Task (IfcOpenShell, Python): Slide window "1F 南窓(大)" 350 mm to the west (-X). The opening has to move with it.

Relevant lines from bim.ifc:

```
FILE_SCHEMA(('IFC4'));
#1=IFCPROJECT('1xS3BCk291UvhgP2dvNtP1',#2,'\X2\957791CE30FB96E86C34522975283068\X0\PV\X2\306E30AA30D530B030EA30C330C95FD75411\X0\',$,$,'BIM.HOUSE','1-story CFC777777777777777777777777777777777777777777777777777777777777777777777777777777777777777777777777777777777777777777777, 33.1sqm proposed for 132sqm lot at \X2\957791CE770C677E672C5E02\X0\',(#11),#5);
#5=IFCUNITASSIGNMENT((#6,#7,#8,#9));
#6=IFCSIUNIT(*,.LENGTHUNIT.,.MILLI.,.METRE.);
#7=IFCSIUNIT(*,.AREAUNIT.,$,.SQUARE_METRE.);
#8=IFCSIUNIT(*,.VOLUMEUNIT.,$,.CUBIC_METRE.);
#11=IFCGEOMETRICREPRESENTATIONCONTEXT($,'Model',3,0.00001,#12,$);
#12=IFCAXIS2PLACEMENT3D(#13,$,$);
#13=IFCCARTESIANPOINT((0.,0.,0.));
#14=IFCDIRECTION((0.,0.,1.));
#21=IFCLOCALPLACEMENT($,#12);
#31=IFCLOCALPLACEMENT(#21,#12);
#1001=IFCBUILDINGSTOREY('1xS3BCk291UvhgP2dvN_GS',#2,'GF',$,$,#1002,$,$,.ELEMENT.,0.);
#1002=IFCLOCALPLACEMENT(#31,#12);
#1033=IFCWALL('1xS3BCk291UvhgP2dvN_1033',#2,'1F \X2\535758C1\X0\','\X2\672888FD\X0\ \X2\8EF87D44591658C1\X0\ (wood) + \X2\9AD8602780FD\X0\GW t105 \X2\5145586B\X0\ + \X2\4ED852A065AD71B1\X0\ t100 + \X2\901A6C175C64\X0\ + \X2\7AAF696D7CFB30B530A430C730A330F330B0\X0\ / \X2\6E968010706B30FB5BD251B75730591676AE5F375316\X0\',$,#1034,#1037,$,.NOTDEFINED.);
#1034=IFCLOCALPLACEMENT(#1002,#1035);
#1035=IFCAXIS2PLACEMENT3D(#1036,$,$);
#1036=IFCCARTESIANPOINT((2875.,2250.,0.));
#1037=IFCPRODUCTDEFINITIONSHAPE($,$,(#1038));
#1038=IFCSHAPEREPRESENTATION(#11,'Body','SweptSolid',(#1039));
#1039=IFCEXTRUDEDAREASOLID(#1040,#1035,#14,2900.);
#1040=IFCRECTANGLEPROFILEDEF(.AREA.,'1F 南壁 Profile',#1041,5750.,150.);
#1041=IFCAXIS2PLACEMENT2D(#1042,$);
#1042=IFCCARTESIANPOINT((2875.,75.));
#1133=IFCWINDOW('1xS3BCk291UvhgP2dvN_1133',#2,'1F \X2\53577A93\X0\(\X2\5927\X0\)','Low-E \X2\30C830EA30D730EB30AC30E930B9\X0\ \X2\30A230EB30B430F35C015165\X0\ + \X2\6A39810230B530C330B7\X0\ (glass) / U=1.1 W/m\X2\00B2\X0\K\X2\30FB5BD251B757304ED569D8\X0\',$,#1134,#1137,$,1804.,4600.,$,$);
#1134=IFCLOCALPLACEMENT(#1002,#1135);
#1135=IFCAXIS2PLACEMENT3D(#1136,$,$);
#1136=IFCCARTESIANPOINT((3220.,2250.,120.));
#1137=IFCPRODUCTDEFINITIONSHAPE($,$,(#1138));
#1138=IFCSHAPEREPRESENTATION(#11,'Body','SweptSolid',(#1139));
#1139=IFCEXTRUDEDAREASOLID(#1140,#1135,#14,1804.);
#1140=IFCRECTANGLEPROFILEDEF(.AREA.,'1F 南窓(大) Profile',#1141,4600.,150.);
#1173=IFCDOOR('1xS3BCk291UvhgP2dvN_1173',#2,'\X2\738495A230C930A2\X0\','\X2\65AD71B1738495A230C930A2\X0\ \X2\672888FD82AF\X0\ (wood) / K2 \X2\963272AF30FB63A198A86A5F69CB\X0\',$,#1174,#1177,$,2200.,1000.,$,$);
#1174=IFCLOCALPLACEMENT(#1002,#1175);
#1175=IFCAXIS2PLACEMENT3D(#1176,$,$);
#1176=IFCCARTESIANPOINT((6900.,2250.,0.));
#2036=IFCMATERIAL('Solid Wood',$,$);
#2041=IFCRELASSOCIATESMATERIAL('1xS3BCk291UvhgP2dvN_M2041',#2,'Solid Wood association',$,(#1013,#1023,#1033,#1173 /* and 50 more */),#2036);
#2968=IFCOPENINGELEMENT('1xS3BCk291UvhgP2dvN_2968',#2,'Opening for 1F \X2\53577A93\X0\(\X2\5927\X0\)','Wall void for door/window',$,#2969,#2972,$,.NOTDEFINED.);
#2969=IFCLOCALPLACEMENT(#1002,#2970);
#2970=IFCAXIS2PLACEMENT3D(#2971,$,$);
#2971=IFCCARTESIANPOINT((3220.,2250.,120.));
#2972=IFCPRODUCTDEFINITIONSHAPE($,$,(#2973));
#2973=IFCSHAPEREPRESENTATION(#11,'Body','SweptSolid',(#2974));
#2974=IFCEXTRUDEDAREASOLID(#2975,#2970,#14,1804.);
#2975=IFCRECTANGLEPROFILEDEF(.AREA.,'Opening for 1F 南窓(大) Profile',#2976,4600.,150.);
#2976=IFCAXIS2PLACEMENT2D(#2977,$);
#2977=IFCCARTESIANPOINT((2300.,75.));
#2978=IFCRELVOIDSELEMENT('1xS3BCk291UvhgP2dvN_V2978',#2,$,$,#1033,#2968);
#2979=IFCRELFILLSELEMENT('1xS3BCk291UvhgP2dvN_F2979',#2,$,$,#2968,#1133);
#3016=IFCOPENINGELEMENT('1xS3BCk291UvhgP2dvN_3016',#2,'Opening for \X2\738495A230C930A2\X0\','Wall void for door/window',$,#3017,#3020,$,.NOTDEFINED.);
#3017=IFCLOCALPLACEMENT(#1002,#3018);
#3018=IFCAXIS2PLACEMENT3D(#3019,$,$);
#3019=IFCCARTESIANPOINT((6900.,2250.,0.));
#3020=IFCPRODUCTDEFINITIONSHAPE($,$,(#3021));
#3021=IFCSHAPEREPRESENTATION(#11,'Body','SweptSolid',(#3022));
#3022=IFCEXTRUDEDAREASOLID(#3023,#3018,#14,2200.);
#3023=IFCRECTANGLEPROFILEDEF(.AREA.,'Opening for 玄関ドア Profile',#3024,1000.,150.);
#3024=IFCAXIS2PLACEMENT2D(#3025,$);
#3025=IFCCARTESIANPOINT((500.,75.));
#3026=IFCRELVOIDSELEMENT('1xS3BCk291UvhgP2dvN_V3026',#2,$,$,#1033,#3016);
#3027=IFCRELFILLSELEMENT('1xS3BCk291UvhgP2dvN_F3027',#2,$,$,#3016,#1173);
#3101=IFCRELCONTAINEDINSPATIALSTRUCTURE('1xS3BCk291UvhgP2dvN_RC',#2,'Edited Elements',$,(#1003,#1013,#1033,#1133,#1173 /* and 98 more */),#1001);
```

```python
import ifcopenshell
import ifcopenshell.api.geometry
import ifcopenshell.util.placement

model = ifcopenshell.open("bim.ifc")

window = model.by_guid("1xS3BCk291UvhgP2dvN_1133")
opening = window.FillsVoids[0].RelatingOpeningElement
wall = opening.VoidsElements[0].RelatingBuildingElement

wall_matrix = ifcopenshell.util.placement.get_local_placement(wall.ObjectPlacement)
shift = wall_matrix[:3, 0] * -350.0
before = ifcopenshell.util.placement.get_local_placement(window.ObjectPlacement)[:3, 3].copy()

# The window is not placed relative to its opening, so move both.
for product in (opening, window):
    matrix = ifcopenshell.util.placement.get_local_placement(product.ObjectPlacement)
    matrix[:3, 3] += shift
    ifcopenshell.api.geometry.edit_object_placement(model, product=product, matrix=matrix, is_si=False)

after = ifcopenshell.util.placement.get_local_placement(window.ObjectPlacement)[:3, 3]
print("window moved by", (after - before).round(3) + 0.0)

model.write("bim-out.ifc")
```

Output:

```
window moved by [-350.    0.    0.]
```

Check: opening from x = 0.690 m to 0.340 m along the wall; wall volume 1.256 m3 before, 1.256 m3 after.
